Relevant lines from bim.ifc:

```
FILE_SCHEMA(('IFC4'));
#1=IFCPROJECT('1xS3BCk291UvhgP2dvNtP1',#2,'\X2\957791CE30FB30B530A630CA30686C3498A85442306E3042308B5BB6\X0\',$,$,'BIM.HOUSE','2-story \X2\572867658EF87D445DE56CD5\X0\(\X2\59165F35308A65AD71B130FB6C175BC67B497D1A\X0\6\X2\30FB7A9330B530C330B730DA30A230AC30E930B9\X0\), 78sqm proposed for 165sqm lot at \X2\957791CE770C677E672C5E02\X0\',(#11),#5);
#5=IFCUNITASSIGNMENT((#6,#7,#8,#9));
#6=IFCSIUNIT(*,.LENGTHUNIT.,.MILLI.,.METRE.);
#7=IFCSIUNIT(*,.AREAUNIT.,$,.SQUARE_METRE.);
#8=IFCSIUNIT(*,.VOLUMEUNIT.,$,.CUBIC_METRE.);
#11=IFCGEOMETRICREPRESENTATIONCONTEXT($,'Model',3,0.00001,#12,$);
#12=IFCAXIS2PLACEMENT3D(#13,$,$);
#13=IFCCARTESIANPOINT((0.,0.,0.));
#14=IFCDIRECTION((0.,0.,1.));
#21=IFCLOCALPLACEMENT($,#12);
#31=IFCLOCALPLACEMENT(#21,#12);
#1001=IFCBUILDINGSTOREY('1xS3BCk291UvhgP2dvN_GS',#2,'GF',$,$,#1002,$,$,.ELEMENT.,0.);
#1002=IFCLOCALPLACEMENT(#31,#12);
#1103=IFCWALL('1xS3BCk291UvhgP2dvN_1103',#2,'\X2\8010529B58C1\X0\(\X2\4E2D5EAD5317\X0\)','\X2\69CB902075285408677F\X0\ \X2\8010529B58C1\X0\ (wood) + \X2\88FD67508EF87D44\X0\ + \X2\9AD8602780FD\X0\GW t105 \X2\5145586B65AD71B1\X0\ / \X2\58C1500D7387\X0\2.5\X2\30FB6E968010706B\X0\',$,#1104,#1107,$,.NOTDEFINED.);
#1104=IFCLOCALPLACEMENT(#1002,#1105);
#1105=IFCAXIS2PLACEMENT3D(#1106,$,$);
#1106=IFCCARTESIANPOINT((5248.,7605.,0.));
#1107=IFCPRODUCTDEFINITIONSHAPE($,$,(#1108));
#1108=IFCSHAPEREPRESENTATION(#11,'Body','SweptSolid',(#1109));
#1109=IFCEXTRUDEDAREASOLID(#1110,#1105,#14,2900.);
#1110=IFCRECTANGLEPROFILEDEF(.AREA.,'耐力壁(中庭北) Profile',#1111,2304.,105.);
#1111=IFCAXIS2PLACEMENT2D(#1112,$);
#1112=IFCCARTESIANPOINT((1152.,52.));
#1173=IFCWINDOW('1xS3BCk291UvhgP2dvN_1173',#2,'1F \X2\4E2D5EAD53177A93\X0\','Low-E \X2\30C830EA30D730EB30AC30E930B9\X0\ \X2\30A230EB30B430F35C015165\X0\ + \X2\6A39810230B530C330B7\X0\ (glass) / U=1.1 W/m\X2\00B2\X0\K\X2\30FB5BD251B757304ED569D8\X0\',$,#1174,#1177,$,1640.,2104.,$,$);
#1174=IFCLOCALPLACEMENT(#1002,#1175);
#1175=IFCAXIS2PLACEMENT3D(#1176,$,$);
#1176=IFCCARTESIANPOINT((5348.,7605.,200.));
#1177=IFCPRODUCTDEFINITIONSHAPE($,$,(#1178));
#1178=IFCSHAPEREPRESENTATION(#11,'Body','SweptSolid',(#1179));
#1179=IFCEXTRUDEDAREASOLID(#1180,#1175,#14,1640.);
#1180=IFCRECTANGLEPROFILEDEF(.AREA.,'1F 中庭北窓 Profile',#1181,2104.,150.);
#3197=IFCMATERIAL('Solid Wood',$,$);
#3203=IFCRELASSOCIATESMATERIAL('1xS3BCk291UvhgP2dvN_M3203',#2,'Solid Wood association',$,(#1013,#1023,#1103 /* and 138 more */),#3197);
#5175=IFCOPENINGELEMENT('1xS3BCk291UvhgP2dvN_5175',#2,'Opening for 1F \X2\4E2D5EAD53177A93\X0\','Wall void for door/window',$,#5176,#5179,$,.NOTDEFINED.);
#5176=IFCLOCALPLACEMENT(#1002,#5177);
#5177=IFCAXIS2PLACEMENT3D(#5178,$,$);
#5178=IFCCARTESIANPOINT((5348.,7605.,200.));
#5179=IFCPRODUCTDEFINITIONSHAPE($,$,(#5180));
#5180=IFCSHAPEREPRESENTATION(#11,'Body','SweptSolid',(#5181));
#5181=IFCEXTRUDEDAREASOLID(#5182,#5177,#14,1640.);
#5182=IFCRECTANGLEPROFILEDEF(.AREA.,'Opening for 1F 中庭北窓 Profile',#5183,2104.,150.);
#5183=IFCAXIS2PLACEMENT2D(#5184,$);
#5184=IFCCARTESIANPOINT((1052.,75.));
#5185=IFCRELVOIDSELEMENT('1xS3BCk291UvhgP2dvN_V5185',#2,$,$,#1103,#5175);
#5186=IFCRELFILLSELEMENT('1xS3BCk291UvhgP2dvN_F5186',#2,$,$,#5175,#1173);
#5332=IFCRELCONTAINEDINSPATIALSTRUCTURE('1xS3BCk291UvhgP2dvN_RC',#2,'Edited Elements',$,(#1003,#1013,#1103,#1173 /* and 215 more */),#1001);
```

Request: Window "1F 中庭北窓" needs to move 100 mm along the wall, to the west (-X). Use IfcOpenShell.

```python
import ifcopenshell
import ifcopenshell.api.geometry
import ifcopenshell.util.placement
import ifcopenshell.util.unit

model = ifcopenshell.open("bim.ifc")
unit_scale = ifcopenshell.util.unit.calculate_unit_scale(model)

window = model.by_guid("1xS3BCk291UvhgP2dvN_1173")
opening = window.FillsVoids[0].RelatingOpeningElement
wall = opening.VoidsElements[0].RelatingBuildingElement

wall_matrix = ifcopenshell.util.placement.get_local_placement(wall.ObjectPlacement)
shift = wall_matrix[:3, 0] * -0.1 / unit_scale
before = ifcopenshell.util.placement.get_local_placement(window.ObjectPlacement)[:3, 3].copy()

# The window is not placed relative to its opening, so move both.
for product in (opening, window):
    matrix = ifcopenshell.util.placement.get_local_placement(product.ObjectPlacement)
    matrix[:3, 3] += shift
    ifcopenshell.api.geometry.edit_object_placement(model, product=product, matrix=matrix, is_si=False)

after = ifcopenshell.util.placement.get_local_placement(window.ObjectPlacement)[:3, 3]
print("window moved by", (after - before).round(3) + 0.0)

model.write("bim_rev.ifc")
```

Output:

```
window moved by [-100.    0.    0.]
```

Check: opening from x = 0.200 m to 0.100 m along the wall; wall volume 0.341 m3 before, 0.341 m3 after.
